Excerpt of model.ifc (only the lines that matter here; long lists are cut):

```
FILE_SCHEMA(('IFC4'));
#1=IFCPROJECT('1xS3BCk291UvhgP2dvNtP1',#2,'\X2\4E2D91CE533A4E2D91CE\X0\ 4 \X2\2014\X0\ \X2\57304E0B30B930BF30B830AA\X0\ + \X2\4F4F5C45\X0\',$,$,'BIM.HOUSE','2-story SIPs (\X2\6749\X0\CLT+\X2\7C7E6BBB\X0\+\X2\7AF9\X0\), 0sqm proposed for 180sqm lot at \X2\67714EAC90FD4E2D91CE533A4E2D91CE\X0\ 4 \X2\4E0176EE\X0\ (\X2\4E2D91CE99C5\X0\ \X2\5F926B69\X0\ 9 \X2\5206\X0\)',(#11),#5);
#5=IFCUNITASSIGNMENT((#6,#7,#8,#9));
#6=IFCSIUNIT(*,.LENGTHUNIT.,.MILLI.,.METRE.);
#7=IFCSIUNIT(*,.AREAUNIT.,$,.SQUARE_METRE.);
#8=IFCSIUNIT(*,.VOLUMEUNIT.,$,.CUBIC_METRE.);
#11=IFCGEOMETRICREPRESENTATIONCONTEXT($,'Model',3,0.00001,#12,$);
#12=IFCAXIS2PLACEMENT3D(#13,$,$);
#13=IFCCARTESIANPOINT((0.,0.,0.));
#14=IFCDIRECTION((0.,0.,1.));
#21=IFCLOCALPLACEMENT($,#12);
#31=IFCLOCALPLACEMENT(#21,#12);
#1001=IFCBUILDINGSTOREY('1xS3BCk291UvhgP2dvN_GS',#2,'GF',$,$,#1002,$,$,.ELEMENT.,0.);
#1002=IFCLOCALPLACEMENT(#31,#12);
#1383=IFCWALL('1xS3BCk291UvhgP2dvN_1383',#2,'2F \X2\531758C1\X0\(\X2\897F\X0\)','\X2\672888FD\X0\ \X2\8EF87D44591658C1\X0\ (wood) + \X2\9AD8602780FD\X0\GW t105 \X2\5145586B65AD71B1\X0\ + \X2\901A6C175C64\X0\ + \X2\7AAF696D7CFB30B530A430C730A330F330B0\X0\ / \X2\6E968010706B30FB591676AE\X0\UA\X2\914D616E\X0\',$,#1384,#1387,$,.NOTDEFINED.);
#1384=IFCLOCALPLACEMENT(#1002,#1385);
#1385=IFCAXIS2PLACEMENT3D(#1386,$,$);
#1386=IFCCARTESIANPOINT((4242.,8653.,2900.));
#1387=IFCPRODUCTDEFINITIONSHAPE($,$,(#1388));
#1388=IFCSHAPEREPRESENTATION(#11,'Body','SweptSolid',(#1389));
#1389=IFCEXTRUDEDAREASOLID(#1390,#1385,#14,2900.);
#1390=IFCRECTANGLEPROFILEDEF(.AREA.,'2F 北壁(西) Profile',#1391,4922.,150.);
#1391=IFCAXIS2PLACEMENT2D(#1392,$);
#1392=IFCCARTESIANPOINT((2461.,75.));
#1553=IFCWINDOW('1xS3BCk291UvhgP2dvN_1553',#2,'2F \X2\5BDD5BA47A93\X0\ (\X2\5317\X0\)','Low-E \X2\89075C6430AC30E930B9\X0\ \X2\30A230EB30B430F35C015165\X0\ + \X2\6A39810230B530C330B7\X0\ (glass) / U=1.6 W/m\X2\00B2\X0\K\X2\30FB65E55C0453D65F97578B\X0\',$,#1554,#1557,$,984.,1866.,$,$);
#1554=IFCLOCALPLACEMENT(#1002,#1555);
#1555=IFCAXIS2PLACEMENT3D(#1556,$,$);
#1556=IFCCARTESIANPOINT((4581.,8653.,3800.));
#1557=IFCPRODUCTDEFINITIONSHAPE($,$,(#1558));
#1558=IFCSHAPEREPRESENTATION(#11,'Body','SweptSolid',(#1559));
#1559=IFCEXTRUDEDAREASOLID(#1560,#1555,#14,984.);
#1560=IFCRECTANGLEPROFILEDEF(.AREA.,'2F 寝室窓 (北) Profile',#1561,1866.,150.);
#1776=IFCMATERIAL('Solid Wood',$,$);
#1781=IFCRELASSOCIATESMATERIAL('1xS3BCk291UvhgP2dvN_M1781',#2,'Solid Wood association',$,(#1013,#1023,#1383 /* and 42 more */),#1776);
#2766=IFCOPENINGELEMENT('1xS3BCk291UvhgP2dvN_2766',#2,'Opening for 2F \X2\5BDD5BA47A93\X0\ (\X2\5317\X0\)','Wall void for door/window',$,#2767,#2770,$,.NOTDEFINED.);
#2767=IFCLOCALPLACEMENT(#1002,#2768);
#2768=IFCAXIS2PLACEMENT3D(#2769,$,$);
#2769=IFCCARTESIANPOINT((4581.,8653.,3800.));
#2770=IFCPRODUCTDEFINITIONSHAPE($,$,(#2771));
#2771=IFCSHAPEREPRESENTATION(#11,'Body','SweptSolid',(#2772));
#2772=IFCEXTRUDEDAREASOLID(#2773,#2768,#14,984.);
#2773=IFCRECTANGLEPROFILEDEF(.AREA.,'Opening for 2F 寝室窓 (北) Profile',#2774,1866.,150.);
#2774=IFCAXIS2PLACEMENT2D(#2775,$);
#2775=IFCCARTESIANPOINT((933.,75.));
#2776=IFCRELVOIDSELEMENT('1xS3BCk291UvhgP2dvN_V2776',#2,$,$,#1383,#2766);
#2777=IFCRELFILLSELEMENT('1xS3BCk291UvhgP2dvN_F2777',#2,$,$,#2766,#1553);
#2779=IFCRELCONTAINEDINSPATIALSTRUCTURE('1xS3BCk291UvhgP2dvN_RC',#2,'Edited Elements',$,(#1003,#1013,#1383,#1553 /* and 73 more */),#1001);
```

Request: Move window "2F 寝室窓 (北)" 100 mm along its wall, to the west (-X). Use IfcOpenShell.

```python
import ifcopenshell
import ifcopenshell.api.geometry
import ifcopenshell.util.placement
import ifcopenshell.util.unit

model = ifcopenshell.open("model.ifc")
unit_scale = ifcopenshell.util.unit.calculate_unit_scale(model)

window = model.by_id(1553)
opening = window.FillsVoids[0].RelatingOpeningElement
wall = opening.VoidsElements[0].RelatingBuildingElement

wall_matrix = ifcopenshell.util.placement.get_local_placement(wall.ObjectPlacement)
shift = wall_matrix[:3, 0] * -0.1 / unit_scale
before = ifcopenshell.util.placement.get_local_placement(window.ObjectPlacement)[:3, 3].copy()

# The window is not placed relative to its opening, so move both.
for product in (opening, window):
    matrix = ifcopenshell.util.placement.get_local_placement(product.ObjectPlacement)
    matrix[:3, 3] += shift
    ifcopenshell.api.geometry.edit_object_placement(model, product=product, matrix=matrix, is_si=False)

after = ifcopenshell.util.placement.get_local_placement(window.ObjectPlacement)[:3, 3]
print("window moved by", (after - before).round(3) + 0.0)

model.write("model-out.ifc")
```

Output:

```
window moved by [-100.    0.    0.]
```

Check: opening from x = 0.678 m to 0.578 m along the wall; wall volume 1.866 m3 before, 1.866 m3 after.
